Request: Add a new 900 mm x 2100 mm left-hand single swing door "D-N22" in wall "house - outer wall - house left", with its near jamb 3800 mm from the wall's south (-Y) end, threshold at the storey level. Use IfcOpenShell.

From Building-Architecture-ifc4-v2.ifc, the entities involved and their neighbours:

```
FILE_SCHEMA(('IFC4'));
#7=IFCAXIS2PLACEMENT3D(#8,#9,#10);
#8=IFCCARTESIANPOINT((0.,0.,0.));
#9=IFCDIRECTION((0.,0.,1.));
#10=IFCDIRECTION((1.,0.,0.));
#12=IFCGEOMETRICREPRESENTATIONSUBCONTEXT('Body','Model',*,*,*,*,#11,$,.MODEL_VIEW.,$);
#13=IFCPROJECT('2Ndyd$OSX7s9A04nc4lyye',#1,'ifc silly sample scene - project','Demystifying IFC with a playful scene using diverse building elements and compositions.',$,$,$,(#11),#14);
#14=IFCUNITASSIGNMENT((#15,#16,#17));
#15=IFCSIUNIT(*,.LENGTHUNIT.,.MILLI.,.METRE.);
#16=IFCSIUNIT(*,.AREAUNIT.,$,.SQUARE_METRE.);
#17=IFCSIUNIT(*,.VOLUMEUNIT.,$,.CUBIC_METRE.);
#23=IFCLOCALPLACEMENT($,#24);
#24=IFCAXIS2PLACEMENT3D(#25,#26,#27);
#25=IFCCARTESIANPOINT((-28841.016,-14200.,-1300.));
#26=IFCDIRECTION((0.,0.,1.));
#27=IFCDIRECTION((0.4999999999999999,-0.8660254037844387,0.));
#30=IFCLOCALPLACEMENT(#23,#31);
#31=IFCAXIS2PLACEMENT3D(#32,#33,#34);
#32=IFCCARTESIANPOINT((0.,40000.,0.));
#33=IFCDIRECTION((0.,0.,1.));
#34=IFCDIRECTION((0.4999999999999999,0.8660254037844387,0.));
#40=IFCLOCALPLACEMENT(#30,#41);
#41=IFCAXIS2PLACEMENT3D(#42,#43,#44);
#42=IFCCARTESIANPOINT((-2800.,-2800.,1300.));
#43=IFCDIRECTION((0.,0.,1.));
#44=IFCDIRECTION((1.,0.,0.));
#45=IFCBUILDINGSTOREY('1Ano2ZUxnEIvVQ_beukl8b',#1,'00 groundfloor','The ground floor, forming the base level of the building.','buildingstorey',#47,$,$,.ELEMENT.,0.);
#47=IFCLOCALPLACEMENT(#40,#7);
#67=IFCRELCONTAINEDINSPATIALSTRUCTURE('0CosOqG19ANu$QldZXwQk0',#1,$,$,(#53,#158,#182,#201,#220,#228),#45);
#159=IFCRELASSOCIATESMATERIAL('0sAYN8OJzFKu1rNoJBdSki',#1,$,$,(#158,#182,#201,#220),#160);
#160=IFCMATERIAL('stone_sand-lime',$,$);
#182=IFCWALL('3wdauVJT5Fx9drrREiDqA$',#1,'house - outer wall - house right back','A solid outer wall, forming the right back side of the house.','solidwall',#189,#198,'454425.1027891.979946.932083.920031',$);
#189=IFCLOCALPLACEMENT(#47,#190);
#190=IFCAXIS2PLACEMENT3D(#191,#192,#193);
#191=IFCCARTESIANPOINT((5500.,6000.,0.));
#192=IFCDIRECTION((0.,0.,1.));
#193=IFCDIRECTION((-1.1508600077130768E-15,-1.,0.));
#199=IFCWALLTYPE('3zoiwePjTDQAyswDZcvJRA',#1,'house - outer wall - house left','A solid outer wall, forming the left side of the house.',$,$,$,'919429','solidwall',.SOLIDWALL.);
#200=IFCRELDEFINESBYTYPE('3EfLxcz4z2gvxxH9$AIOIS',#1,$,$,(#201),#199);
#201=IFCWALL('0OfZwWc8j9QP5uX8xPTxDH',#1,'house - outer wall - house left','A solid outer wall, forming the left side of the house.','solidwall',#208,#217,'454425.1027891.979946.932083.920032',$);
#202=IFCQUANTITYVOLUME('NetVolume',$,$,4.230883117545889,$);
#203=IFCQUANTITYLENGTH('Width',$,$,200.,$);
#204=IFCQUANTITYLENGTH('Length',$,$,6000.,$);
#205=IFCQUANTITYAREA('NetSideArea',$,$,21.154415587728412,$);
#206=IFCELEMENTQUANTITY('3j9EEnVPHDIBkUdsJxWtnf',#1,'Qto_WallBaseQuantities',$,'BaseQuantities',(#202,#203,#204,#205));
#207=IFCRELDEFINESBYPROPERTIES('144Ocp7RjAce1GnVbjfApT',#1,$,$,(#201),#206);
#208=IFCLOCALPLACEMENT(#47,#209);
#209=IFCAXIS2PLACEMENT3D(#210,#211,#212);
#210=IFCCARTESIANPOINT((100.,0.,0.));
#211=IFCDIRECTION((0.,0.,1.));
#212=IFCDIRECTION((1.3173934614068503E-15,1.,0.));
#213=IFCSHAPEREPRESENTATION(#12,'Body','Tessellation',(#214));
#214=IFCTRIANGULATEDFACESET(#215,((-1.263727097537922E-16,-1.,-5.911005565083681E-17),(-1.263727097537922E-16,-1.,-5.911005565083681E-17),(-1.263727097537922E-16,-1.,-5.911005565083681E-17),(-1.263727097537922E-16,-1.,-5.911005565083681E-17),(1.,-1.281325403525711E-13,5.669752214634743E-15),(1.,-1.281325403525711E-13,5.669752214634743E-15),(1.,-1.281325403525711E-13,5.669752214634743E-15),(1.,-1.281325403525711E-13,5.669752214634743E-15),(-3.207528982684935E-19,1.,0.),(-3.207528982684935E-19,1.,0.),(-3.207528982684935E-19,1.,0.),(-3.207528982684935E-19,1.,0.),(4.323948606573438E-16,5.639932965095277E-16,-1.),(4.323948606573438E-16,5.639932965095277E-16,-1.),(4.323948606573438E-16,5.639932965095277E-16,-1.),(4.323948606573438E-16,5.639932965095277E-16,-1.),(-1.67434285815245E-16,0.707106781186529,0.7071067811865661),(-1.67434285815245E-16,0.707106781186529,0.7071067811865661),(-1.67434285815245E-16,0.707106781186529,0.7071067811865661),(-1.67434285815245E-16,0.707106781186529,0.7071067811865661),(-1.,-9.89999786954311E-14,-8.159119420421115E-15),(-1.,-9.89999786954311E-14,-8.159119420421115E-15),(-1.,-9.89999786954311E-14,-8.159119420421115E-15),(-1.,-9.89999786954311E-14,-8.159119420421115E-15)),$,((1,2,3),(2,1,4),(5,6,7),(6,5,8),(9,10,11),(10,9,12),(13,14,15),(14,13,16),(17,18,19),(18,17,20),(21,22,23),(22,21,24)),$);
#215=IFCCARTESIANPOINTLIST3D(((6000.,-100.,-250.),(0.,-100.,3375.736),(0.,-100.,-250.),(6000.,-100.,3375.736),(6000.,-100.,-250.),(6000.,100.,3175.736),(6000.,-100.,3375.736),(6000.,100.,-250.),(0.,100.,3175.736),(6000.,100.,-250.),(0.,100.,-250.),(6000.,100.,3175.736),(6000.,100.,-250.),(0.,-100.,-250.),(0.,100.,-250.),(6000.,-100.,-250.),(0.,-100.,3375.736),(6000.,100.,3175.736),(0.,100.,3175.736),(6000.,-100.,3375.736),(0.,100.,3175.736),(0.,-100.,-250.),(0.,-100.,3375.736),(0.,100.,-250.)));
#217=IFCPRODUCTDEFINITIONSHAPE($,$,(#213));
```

```python
import numpy as np
import ifcopenshell
import ifcopenshell.api.feature
import ifcopenshell.api.geometry
import ifcopenshell.api.pset
import ifcopenshell.api.root
import ifcopenshell.api.spatial
import ifcopenshell.geom
import ifcopenshell.util.element
import ifcopenshell.util.placement
import ifcopenshell.util.representation
import ifcopenshell.util.shape
import ifcopenshell.util.unit

model = ifcopenshell.open("Building-Architecture-ifc4-v2.ifc")
unit_scale = ifcopenshell.util.unit.calculate_unit_scale(model)
area_scale = ifcopenshell.util.unit.calculate_unit_scale(model, "AREAUNIT")
volume_scale = ifcopenshell.util.unit.calculate_unit_scale(model, "VOLUMEUNIT")
settings = ifcopenshell.geom.settings()


def volume(element):
    """Net volume in cubic metres, openings subtracted."""
    shape = ifcopenshell.geom.create_shape(settings, element)
    return ifcopenshell.util.shape.get_volume(shape.geometry)


wall = model.by_guid("0OfZwWc8j9QP5uX8xPTxDH")
storey = ifcopenshell.util.element.get_container(wall, ifc_class="IfcBuildingStorey")
context = ifcopenshell.util.representation.get_context(model, "Model", "Body", "MODEL_VIEW")
before = volume(wall)

width, height, from_end, sill = 0.9, 2.1, 3.8, 0.0  # metres

# The wall runs along its own X axis, and the end named is its -X end.
wall_shape = ifcopenshell.geom.create_shape(settings, wall)
x, y, z = ifcopenshell.util.shape.get_vertices(wall_shape.geometry).T
start = x.min() + from_end
face, thickness = float(y.min()), float(y.max() - y.min())
wall_matrix = ifcopenshell.util.placement.get_local_placement(wall.ObjectPlacement)
level = ifcopenshell.util.placement.get_local_placement(storey.ObjectPlacement)[2, 3]


def in_wall(x, y):
    """Placement at x, y metres in the wall's axes, at sill height."""
    matrix = wall_matrix.copy()
    matrix[:, 3] = wall_matrix @ np.array([x / unit_scale, y / unit_scale, 0.0, 1.0])
    matrix[2, 3] = level + sill / unit_scale
    return matrix


# Opening: a box that overshoots both wall faces by 50 mm.
opening = ifcopenshell.api.root.create_entity(model, ifc_class="IfcOpeningElement", predefined_type="OPENING")
box = ifcopenshell.api.geometry.add_wall_representation(
    model, context=context, length=width, height=height, thickness=thickness + 0.1
)
ifcopenshell.api.geometry.assign_representation(model, product=opening, representation=box)
ifcopenshell.api.geometry.edit_object_placement(model, product=opening, matrix=in_wall(start, face - 0.05), is_si=False)
ifcopenshell.api.feature.add_feature(model, feature=opening, element=wall)

door = ifcopenshell.api.root.create_entity(model, ifc_class="IfcDoor", name="D-N22", predefined_type="DOOR")
door.OverallWidth, door.OverallHeight = width / unit_scale, height / unit_scale
door.OperationType = "SINGLE_SWING_LEFT"
body = ifcopenshell.api.geometry.add_door_representation(
    model,
    context=context,
    overall_width=door.OverallWidth,
    overall_height=door.OverallHeight,
    operation_type="SINGLE_SWING_LEFT",
    lining_properties={"LiningDepth": thickness / unit_scale, "ThresholdDepth": thickness / unit_scale},
)
ifcopenshell.api.geometry.assign_representation(model, product=door, representation=body)
ifcopenshell.api.spatial.assign_container(model, products=[door], relating_structure=storey)
ifcopenshell.api.feature.add_filling(model, opening=opening, element=door)

# The lining spans the wall, so the door starts at the wall face.
ifcopenshell.api.geometry.edit_object_placement(model, product=door, matrix=in_wall(start, face), is_si=False)

after = volume(wall)

# Update the wall's stored quantities.
qto = model.by_id(ifcopenshell.util.element.get_pset(wall, "Qto_WallBaseQuantities", should_inherit=False)["id"])
ifcopenshell.api.pset.edit_qto(model, qto=qto, properties={
    "NetVolume": after / volume_scale,
    "NetSideArea": after / thickness / area_scale,
})

print(f"wall volume {before:.3f} -> {after:.3f} m3")

model.write("Building-Architecture-ifc4-v2_v2.ifc")
```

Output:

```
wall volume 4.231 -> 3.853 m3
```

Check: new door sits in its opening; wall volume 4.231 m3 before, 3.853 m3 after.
